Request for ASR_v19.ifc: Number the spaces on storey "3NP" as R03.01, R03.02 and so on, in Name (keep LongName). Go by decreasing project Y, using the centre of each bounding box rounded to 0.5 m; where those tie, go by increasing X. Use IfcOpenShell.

First a look at what the model holds.

```python
import ifcopenshell
import ifcopenshell.util.element
import ifcopenshell.util.placement

model = ifcopenshell.open("ASR_v19.ifc")
print(model.schema)
storey = next(s for s in model.by_type("IfcBuildingStorey") if s.Name == "3NP")
spaces = [e for e in ifcopenshell.util.element.get_decomposition(storey) if e.is_a("IfcSpace")]
for e in sorted(spaces, key=lambda e: e.id()):
    origin = ifcopenshell.util.placement.get_local_placement(e.ObjectPlacement)[:3, 3]
    print(e.id(), e.Name, e.LongName, origin.round(2) + 0.0, sep=" | ")
```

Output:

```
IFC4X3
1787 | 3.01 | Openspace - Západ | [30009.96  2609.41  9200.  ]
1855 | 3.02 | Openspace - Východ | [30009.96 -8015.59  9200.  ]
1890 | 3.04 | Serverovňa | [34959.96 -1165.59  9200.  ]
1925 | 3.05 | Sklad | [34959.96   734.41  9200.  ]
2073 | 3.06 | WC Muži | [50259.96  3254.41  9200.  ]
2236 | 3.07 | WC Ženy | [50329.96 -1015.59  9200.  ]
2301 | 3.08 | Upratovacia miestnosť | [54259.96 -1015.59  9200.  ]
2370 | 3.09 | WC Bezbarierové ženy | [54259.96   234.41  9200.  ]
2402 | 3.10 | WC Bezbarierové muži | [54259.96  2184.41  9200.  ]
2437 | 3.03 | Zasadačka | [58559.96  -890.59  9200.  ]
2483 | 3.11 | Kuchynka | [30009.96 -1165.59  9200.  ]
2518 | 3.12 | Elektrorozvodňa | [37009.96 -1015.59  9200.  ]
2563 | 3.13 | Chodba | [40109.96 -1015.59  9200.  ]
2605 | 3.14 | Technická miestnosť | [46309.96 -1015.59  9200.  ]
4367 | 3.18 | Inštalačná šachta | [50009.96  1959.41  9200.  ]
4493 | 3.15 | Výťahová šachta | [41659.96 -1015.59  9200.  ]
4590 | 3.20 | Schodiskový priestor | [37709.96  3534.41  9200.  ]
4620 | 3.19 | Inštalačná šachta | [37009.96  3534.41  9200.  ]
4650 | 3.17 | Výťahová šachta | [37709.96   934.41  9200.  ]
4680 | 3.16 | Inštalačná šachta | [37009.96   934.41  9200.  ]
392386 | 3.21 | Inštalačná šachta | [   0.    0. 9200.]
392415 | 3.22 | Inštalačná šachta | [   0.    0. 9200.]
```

```python
import ifcopenshell
import ifcopenshell.geom
import ifcopenshell.util.element
import ifcopenshell.util.shape

model = ifcopenshell.open("ASR_v19.ifc")
settings = ifcopenshell.geom.settings()
settings.set("use-world-coords", True)


def centre(element):
    shape = ifcopenshell.geom.create_shape(settings, element)
    return ifcopenshell.util.shape.get_bbox_centroid(shape.geometry)


storey = next(s for s in model.by_type("IfcBuildingStorey") if s.Name == "3NP")
spaces = [e for e in ifcopenshell.util.element.get_decomposition(storey) if e.is_a("IfcSpace")]

# Insertion points can sit at a corner or the storey origin, so sort by the geometry (in metres).
centres = {e: centre(e) for e in spaces}
spaces.sort(key=lambda e: (-round(centres[e][1] / 0.5), centres[e][0]))

for i, e in enumerate(spaces, start=1):
    number = f"R03.{i:02d}"
    e.Name = number
    print(e.id(), number)

model.write("ASR_v19_rev.ifc")
```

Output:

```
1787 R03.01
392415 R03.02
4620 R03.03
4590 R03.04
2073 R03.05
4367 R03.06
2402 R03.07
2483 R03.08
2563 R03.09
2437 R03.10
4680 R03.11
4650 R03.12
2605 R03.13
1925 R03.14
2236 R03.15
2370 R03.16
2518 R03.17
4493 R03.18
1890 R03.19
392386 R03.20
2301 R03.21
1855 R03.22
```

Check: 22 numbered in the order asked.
